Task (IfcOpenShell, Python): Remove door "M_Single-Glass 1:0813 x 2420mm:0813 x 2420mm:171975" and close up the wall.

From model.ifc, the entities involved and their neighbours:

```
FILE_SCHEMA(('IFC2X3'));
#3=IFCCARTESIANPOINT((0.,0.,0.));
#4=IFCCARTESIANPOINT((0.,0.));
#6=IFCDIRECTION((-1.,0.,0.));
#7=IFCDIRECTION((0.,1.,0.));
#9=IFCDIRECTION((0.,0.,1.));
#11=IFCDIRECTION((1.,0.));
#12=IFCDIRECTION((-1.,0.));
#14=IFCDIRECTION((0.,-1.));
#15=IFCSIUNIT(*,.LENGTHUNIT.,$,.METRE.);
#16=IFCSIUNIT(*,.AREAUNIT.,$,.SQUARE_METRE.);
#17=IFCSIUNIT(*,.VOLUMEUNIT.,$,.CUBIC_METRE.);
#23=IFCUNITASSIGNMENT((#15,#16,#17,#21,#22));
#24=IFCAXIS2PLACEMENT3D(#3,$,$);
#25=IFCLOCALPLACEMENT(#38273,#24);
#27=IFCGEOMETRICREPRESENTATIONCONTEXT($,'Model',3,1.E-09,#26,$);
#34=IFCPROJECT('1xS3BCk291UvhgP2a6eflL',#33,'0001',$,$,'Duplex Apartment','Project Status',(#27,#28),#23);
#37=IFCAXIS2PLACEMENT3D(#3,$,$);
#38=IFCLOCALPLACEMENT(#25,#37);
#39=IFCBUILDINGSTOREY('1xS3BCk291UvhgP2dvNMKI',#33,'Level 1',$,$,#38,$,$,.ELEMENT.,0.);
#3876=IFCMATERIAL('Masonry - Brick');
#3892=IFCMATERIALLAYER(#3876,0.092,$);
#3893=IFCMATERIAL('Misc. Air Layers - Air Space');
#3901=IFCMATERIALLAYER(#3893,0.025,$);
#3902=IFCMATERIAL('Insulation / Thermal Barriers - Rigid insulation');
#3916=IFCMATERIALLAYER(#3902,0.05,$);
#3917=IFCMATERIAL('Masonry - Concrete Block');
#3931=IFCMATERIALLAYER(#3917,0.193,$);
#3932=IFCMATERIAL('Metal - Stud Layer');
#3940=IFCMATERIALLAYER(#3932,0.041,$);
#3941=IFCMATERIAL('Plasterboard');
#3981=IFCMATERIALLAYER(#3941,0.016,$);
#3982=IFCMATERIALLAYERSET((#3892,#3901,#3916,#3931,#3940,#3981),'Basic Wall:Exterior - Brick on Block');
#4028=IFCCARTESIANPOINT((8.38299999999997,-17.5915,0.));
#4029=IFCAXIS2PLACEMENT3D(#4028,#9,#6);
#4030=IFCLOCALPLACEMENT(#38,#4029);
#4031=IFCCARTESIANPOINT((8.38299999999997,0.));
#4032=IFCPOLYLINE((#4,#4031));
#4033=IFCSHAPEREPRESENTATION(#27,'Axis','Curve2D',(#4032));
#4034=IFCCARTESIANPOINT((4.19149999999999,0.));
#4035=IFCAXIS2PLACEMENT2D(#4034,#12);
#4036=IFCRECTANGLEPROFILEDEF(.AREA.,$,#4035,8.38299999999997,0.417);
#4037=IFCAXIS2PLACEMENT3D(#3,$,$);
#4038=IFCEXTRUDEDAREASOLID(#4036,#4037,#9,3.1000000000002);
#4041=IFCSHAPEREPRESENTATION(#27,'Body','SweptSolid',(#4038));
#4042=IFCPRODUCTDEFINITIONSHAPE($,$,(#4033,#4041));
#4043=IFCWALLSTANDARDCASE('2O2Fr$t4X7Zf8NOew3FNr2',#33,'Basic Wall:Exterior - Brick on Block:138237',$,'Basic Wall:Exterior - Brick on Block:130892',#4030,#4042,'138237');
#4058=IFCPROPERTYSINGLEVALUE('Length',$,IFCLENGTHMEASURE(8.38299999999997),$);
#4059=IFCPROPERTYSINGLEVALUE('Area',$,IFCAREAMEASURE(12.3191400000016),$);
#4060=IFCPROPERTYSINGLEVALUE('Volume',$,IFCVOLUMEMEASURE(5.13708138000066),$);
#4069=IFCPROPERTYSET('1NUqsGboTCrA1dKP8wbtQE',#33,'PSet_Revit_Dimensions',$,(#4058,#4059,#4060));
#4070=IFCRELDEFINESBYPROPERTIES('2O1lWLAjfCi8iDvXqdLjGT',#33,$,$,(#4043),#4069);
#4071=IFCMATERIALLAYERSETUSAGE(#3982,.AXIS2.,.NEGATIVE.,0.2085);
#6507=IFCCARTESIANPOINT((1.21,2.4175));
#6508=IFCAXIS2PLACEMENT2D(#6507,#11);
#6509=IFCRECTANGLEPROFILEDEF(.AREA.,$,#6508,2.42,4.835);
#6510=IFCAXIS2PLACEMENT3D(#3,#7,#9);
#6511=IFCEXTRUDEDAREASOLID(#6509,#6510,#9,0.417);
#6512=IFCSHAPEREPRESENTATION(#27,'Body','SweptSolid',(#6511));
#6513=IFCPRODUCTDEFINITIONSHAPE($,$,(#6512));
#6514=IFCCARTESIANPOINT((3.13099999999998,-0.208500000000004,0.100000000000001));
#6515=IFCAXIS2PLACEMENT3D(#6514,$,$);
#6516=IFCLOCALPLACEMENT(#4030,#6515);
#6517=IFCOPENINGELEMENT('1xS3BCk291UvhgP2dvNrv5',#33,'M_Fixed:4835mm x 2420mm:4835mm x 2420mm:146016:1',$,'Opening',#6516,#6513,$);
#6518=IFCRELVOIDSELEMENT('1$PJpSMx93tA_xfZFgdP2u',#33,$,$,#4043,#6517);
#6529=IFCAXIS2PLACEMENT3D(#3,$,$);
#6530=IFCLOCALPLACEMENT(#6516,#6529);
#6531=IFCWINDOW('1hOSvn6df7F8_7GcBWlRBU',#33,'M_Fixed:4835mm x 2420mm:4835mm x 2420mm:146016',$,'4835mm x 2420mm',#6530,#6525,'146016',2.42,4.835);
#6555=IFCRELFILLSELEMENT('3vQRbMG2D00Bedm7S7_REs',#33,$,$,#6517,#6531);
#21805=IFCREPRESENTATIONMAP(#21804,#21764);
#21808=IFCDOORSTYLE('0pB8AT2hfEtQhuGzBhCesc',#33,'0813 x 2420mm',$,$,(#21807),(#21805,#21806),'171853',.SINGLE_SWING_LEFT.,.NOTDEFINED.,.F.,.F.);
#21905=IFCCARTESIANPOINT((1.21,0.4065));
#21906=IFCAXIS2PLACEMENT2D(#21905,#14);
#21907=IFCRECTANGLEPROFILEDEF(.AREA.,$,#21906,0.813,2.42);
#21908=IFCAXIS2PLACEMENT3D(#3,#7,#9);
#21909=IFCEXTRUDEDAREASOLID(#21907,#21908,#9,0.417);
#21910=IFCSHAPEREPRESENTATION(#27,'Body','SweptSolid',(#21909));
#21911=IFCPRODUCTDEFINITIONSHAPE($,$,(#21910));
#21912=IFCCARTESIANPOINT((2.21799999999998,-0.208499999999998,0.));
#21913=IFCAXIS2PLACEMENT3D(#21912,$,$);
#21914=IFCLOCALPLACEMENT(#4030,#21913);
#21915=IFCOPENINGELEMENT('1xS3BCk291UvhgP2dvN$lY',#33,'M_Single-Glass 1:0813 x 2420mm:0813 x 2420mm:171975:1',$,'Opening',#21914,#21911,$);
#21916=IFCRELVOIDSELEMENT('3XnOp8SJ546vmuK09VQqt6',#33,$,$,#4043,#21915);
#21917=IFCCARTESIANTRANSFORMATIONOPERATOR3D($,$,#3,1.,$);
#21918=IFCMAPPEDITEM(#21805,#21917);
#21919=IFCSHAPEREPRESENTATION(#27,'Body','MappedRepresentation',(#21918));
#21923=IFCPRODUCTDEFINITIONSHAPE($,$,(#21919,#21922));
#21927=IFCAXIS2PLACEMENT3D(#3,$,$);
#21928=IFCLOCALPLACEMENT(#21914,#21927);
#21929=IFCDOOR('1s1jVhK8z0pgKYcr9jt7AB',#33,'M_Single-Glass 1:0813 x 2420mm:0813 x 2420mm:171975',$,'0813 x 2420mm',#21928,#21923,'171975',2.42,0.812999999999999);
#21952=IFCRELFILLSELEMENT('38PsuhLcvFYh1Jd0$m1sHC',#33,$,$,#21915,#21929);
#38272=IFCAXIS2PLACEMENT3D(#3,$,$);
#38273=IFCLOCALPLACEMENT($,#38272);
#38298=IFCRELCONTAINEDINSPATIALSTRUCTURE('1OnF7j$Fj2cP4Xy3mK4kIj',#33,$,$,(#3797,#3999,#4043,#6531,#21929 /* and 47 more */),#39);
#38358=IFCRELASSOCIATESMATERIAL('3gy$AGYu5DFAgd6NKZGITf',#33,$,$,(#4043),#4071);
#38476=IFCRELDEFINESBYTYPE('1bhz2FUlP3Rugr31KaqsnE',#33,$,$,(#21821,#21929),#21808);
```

```python
import ifcopenshell
import ifcopenshell.api.feature
import ifcopenshell.api.pset
import ifcopenshell.api.root
import ifcopenshell.geom
import ifcopenshell.util.element
import ifcopenshell.util.shape
import ifcopenshell.util.unit

model = ifcopenshell.open("model.ifc")
area_scale = ifcopenshell.util.unit.calculate_unit_scale(model, "AREAUNIT")
volume_scale = ifcopenshell.util.unit.calculate_unit_scale(model, "VOLUMEUNIT")
settings = ifcopenshell.geom.settings()


def volume(element):
    """Net volume in cubic metres, openings subtracted."""
    shape = ifcopenshell.geom.create_shape(settings, element)
    return ifcopenshell.util.shape.get_volume(shape.geometry)


door = model.by_guid("1s1jVhK8z0pgKYcr9jt7AB")
opening = door.FillsVoids[0].RelatingOpeningElement
wall = opening.VoidsElements[0].RelatingBuildingElement
before = volume(wall)

ifcopenshell.api.root.remove_product(model, product=door)
ifcopenshell.api.feature.remove_feature(model, feature=opening)

after = volume(wall)
thickness = 0.417  # wall thickness in metres

# Update the wall's stored quantities.
pset = model.by_id(ifcopenshell.util.element.get_pset(wall, "PSet_Revit_Dimensions", should_inherit=False)["id"])
ifcopenshell.api.pset.edit_pset(model, pset=pset, properties={
    "Area": model.create_entity("IfcAreaMeasure", after / thickness / area_scale),
    "Volume": model.create_entity("IfcVolumeMeasure", after / volume_scale),
})

print(f"wall volume {before:.3f} -> {after:.3f} m3")

model.write("model_edited.ifc")
```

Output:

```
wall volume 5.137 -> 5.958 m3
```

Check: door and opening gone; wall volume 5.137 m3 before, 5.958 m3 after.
